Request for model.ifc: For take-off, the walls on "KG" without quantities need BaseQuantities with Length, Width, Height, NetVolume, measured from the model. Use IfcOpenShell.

First a look at what the model holds.

```python
import ifcopenshell
import ifcopenshell.util.element
import ifcopenshell.util.unit

model = ifcopenshell.open("model.ifc")
print(model.schema)
for unit_type in ("LENGTHUNIT", "AREAUNIT", "VOLUMEUNIT"):
    print(unit_type, ifcopenshell.util.unit.calculate_unit_scale(model, unit_type))
storey = next(s for s in model.by_type("IfcBuildingStorey") if s.Name == "KG")
walls = [e for e in ifcopenshell.util.element.get_decomposition(storey) if e.is_a("IfcWall")]
for e in sorted(walls, key=lambda e: e.id()):
    print(e.id(), e.is_a(), e.Name, list(ifcopenshell.util.element.get_psets(e, qtos_only=True)), sep=" | ")
```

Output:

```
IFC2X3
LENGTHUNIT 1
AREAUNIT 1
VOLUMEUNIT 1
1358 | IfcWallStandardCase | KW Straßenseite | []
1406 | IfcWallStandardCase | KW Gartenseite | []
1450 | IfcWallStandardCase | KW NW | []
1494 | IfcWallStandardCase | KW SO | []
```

```python
import ifcopenshell
import ifcopenshell.api.pset
import ifcopenshell.geom
import ifcopenshell.util.element
import ifcopenshell.util.shape
import ifcopenshell.util.unit

model = ifcopenshell.open("model.ifc")
unit_scale = ifcopenshell.util.unit.calculate_unit_scale(model)
volume_scale = ifcopenshell.util.unit.calculate_unit_scale(model, "VOLUMEUNIT")
settings = ifcopenshell.geom.settings()

storey = next(s for s in model.by_type("IfcBuildingStorey") if s.Name == "KG")
walls = [e for e in ifcopenshell.util.element.get_decomposition(storey) if e.is_a("IfcWall")]

for e in sorted(walls, key=lambda e: e.id()):
    if ifcopenshell.util.element.get_psets(e, qtos_only=True, should_inherit=False):
        continue
    # Geometry comes back in metres, in the element's own axes.
    shape = ifcopenshell.geom.create_shape(settings, e)
    values = {
        "Length": ifcopenshell.util.shape.get_x(shape.geometry) / unit_scale,
        "Width": ifcopenshell.util.shape.get_y(shape.geometry) / unit_scale,
        "Height": ifcopenshell.util.shape.get_z(shape.geometry) / unit_scale,
        "NetVolume": ifcopenshell.util.shape.get_volume(shape.geometry) / volume_scale,
    }
    qto = ifcopenshell.api.pset.add_qto(model, product=e, name="BaseQuantities")
    ifcopenshell.api.pset.edit_qto(model, qto=qto, properties=values)
    print(e.id(), {k: round(v, 3) for k, v in values.items()})

model.write("model_rev.ifc")
```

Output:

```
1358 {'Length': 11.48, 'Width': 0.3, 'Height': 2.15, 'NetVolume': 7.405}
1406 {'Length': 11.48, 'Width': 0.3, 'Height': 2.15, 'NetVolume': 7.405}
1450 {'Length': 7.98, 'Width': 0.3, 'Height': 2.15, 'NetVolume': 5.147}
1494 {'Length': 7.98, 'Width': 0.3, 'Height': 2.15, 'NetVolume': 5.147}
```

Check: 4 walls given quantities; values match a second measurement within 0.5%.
